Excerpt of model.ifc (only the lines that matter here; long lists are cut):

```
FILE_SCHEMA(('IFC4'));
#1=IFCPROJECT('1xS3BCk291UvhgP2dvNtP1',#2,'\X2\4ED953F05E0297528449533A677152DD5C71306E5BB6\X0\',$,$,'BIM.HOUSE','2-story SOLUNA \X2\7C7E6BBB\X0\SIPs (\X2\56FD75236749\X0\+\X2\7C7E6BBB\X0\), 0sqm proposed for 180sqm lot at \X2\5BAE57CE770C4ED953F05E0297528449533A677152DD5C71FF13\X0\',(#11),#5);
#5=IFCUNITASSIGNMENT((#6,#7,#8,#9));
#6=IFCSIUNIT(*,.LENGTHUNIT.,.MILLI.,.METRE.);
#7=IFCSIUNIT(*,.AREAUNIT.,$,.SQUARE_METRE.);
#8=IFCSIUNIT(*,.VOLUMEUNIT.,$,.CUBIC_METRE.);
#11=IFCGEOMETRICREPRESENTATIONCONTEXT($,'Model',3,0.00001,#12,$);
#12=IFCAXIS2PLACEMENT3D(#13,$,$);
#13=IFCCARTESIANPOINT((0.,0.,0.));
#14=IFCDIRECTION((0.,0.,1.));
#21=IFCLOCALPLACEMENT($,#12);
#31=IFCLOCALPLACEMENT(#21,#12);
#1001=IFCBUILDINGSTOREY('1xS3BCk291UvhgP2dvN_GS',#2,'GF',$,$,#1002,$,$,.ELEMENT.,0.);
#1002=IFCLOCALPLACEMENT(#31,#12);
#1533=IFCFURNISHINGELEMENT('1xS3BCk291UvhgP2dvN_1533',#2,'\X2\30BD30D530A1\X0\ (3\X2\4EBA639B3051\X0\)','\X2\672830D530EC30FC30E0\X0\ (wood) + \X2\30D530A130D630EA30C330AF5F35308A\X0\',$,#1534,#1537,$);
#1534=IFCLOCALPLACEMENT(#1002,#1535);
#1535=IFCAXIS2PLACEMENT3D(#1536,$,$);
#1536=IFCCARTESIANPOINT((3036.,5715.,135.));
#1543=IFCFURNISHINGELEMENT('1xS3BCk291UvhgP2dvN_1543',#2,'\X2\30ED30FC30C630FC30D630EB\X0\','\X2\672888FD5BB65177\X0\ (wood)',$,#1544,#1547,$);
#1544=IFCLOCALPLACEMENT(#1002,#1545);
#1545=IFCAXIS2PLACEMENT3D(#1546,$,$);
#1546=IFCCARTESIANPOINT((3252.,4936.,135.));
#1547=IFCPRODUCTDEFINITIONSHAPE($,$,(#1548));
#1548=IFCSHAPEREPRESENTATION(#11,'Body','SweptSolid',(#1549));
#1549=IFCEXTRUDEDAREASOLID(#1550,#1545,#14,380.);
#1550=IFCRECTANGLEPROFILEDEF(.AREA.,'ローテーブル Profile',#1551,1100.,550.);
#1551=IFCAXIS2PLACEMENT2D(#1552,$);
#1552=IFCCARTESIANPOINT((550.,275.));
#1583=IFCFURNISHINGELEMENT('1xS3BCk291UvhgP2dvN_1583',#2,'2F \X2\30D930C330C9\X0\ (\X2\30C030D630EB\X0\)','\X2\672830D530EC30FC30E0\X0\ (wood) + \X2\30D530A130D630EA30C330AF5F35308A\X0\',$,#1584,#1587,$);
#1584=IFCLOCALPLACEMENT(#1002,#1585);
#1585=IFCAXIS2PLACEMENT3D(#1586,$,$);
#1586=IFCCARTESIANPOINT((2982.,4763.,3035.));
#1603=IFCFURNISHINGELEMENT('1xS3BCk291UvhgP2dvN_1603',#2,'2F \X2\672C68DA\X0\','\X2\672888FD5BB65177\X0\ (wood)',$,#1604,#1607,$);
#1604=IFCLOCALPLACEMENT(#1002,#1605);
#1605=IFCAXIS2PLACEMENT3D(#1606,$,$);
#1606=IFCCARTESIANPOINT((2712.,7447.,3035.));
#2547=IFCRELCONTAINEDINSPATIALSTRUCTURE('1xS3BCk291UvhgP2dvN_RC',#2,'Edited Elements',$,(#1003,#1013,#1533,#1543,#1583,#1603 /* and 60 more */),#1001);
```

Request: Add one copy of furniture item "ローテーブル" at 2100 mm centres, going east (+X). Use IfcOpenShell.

```python
import numpy as np
import ifcopenshell
import ifcopenshell.api.geometry
import ifcopenshell.api.root
import ifcopenshell.util.element
import ifcopenshell.util.placement

model = ifcopenshell.open("model.ifc")


def reuse_history(source, copy):
    """copy_class also copies each property set's owner history, people and application; keep the originals."""
    for rel in copy.IsDefinedBy:
        if rel.is_a("IfcRelDefinesByProperties") and (history := rel.RelatingPropertyDefinition.OwnerHistory):
            rel.RelatingPropertyDefinition.OwnerHistory = source.OwnerHistory
            ifcopenshell.util.element.remove_deep2(model, history)


source = model.by_id(1543)
base = ifcopenshell.util.placement.get_local_placement(source.ObjectPlacement)
step = np.array([1.0, 0.0, 0.0]) * 2100.0

for i in range(1, 2):
    copy = ifcopenshell.api.root.copy_class(model, product=source)
    copy.Representation = ifcopenshell.util.element.copy_deep(
        model, source.Representation, exclude=["IfcGeometricRepresentationContext", "IfcRepresentationMap"]
    )
    reuse_history(source, copy)
    matrix = base.copy()
    matrix[:3, 3] += i * step
    print("added at", matrix[:3, 3].round(3) + 0.0)
    ifcopenshell.api.geometry.edit_object_placement(model, product=copy, matrix=matrix, is_si=False)

model.write("model_v2.ifc")
```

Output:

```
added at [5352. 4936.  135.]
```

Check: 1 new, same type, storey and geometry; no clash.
